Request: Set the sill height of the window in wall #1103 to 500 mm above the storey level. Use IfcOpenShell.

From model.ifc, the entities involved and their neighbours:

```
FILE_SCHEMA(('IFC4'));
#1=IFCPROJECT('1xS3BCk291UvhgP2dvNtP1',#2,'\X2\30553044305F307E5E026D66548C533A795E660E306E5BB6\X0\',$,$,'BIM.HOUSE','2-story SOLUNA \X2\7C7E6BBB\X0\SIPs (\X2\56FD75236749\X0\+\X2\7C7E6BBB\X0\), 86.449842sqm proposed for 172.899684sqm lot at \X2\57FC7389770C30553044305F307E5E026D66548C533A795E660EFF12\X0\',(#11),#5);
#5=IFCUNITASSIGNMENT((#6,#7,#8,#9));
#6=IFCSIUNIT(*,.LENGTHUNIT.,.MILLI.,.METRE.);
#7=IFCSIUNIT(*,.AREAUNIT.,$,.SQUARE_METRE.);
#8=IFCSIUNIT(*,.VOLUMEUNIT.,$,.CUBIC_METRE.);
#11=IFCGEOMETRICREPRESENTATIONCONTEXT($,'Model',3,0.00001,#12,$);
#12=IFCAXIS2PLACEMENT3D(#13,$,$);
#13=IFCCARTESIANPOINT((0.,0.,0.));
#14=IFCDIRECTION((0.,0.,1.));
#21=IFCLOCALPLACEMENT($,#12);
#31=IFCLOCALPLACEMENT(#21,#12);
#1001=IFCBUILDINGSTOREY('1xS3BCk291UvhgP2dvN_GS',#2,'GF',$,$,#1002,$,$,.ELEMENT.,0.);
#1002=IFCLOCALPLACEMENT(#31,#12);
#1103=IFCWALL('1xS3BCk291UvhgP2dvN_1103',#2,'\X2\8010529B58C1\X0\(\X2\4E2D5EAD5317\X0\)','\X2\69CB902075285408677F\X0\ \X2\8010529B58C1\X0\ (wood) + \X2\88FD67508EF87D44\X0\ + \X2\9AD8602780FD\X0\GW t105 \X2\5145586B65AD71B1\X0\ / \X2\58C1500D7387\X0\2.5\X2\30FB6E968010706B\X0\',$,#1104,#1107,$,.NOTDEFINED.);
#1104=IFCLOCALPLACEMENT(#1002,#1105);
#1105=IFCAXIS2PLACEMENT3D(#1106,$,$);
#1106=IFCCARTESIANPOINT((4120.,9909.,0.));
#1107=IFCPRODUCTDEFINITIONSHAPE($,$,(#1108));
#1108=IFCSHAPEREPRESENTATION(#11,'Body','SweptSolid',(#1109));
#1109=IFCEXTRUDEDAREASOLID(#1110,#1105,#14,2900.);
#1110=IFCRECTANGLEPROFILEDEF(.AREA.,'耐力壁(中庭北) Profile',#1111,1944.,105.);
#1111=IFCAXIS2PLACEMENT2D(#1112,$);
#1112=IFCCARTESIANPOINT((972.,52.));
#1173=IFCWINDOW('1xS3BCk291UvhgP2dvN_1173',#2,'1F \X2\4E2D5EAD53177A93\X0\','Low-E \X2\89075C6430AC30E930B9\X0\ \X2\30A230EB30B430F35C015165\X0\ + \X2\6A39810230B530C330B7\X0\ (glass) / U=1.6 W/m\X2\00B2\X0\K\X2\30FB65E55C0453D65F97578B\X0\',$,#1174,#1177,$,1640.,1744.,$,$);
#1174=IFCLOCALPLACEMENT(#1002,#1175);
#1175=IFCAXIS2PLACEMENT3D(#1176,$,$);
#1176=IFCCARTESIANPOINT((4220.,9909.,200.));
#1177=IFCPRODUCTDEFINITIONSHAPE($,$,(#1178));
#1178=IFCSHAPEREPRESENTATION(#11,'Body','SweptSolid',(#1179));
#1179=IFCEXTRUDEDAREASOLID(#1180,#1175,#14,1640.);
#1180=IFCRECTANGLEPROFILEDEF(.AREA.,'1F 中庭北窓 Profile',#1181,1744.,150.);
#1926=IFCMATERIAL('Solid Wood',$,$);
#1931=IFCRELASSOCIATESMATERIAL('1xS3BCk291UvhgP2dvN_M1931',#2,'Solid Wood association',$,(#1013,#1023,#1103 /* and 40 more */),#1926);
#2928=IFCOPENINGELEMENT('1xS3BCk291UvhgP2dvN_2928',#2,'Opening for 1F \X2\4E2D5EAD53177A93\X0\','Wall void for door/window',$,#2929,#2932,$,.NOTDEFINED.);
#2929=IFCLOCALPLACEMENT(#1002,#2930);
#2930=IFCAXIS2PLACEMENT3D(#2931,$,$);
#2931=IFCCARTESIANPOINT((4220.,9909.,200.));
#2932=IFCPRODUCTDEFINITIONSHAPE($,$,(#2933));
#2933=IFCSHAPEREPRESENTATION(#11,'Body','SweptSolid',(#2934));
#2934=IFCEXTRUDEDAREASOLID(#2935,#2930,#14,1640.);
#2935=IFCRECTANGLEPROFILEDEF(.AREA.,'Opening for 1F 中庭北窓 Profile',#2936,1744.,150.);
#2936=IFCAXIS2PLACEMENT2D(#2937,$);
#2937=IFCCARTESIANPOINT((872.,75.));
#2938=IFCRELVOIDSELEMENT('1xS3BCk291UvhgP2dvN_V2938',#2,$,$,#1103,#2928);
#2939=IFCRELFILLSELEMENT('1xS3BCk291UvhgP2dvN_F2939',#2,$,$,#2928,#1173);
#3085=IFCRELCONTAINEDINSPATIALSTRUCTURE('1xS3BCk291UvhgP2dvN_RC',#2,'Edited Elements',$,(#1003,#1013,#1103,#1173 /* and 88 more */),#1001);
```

```python
import numpy as np
import ifcopenshell
import ifcopenshell.api.geometry
import ifcopenshell.geom
import ifcopenshell.util.element
import ifcopenshell.util.placement
import ifcopenshell.util.shape
import ifcopenshell.util.unit

model = ifcopenshell.open("model.ifc")
unit_scale = ifcopenshell.util.unit.calculate_unit_scale(model)

window = model.by_guid("1xS3BCk291UvhgP2dvN_1173")
opening = window.FillsVoids[0].RelatingOpeningElement
storey = ifcopenshell.util.element.get_container(window, ifc_class="IfcBuildingStorey")
level = ifcopenshell.util.placement.get_local_placement(storey.ObjectPlacement)[2, 3]

# The opening's origin need not be at the sill, so measure its lowest point.
shape = ifcopenshell.geom.create_shape(ifcopenshell.geom.settings(), opening)
bottom = ifcopenshell.util.shape.get_shape_bottom_elevation(shape, shape.geometry) / unit_scale
dz = level + 500.0 - bottom

shift = np.array([0.0, 0.0, dz])
# The window is not placed relative to its opening, so move both.
for product in (opening, window):
    matrix = ifcopenshell.util.placement.get_local_placement(product.ObjectPlacement)
    matrix[:3, 3] += shift
    ifcopenshell.api.geometry.edit_object_placement(model, product=product, matrix=matrix, is_si=False)

print(f"moved by {dz * unit_scale:+.3f} m")

model.write("model_edited.ifc")
```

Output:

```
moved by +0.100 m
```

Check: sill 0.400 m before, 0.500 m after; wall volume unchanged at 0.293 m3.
